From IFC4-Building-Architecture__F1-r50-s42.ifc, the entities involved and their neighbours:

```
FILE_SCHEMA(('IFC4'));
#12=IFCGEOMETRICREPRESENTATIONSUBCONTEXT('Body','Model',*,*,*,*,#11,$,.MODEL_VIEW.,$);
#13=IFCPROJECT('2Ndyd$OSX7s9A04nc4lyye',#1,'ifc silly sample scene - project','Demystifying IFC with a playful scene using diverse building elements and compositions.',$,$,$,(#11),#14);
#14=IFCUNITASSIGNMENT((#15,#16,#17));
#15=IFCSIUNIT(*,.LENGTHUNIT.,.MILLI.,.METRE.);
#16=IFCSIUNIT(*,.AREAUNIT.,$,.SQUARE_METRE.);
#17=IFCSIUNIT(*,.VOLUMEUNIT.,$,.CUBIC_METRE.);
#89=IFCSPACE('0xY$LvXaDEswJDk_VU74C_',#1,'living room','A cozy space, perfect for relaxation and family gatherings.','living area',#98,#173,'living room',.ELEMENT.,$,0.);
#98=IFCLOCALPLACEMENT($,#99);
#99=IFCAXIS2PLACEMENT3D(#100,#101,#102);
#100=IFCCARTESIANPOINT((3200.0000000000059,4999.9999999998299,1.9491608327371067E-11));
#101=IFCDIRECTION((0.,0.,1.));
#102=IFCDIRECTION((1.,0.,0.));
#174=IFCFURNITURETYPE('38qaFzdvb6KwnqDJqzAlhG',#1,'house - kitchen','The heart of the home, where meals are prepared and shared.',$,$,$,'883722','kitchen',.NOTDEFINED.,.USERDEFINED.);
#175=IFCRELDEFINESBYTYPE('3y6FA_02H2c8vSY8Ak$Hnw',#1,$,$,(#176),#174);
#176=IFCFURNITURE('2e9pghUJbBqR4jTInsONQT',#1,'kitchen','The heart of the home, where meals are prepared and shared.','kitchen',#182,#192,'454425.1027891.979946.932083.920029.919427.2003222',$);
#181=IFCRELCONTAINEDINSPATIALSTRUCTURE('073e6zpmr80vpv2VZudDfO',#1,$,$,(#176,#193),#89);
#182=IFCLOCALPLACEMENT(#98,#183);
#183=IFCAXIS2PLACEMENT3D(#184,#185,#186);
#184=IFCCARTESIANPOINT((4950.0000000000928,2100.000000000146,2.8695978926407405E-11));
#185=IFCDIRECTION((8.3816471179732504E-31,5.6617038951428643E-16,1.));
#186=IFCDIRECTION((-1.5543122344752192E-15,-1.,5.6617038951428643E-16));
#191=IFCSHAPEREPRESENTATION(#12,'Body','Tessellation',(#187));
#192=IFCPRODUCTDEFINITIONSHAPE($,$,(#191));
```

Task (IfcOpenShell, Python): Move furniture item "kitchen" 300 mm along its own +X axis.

```python
import ifcopenshell
import ifcopenshell.api.geometry
import ifcopenshell.util.placement

model = ifcopenshell.open("IFC4-Building-Architecture__F1-r50-s42.ifc")

item = model.by_guid("2e9pghUJbBqR4jTInsONQT")
matrix = ifcopenshell.util.placement.get_local_placement(item.ObjectPlacement)
matrix[:3, 3] += matrix[:3, 0] * 300.0
ifcopenshell.api.geometry.edit_object_placement(model, product=item, matrix=matrix, is_si=False)

print(ifcopenshell.util.placement.get_local_placement(item.ObjectPlacement).round(3) + 0.0)

model.write("IFC4-Building-Architecture__F1-r50-s42_v2.ifc")
```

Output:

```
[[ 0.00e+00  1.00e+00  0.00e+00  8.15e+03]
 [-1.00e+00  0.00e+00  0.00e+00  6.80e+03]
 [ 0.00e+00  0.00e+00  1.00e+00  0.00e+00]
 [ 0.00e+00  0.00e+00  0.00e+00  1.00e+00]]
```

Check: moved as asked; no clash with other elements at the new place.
